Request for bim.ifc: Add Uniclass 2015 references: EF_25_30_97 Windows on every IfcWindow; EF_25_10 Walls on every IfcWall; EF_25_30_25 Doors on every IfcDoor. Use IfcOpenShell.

First a look at what the model holds.

```python
import ifcopenshell

model = ifcopenshell.open("bim.ifc")
print(model.schema)
print("classifications:", [c.Name for c in model.by_type("IfcClassification")])
for ifc_class in ("IfcDoor", "IfcRoof", "IfcStair", "IfcWall", "IfcWindow"):
    print(ifc_class, len(model.by_type(ifc_class)))
```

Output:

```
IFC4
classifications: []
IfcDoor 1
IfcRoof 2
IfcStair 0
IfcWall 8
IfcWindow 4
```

```python
import ifcopenshell
import ifcopenshell.api.classification

model = ifcopenshell.open("bim.ifc")

system = ifcopenshell.api.classification.add_classification(model, classification="Uniclass 2015")

codes = {
    "IfcWindow": ("EF_25_30_97", "Windows"),
    "IfcWall": ("EF_25_10", "Walls"),
    "IfcDoor": ("EF_25_30_25", "Doors"),
}
for ifc_class, (code, name) in codes.items():
    products = model.by_type(ifc_class)
    ifcopenshell.api.classification.add_reference(
        model, products=products, classification=system, identification=code, name=name
    )
    print(code, len(products))

model.write("bim_rev.ifc")
```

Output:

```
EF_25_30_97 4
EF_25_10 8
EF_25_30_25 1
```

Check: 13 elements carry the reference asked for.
